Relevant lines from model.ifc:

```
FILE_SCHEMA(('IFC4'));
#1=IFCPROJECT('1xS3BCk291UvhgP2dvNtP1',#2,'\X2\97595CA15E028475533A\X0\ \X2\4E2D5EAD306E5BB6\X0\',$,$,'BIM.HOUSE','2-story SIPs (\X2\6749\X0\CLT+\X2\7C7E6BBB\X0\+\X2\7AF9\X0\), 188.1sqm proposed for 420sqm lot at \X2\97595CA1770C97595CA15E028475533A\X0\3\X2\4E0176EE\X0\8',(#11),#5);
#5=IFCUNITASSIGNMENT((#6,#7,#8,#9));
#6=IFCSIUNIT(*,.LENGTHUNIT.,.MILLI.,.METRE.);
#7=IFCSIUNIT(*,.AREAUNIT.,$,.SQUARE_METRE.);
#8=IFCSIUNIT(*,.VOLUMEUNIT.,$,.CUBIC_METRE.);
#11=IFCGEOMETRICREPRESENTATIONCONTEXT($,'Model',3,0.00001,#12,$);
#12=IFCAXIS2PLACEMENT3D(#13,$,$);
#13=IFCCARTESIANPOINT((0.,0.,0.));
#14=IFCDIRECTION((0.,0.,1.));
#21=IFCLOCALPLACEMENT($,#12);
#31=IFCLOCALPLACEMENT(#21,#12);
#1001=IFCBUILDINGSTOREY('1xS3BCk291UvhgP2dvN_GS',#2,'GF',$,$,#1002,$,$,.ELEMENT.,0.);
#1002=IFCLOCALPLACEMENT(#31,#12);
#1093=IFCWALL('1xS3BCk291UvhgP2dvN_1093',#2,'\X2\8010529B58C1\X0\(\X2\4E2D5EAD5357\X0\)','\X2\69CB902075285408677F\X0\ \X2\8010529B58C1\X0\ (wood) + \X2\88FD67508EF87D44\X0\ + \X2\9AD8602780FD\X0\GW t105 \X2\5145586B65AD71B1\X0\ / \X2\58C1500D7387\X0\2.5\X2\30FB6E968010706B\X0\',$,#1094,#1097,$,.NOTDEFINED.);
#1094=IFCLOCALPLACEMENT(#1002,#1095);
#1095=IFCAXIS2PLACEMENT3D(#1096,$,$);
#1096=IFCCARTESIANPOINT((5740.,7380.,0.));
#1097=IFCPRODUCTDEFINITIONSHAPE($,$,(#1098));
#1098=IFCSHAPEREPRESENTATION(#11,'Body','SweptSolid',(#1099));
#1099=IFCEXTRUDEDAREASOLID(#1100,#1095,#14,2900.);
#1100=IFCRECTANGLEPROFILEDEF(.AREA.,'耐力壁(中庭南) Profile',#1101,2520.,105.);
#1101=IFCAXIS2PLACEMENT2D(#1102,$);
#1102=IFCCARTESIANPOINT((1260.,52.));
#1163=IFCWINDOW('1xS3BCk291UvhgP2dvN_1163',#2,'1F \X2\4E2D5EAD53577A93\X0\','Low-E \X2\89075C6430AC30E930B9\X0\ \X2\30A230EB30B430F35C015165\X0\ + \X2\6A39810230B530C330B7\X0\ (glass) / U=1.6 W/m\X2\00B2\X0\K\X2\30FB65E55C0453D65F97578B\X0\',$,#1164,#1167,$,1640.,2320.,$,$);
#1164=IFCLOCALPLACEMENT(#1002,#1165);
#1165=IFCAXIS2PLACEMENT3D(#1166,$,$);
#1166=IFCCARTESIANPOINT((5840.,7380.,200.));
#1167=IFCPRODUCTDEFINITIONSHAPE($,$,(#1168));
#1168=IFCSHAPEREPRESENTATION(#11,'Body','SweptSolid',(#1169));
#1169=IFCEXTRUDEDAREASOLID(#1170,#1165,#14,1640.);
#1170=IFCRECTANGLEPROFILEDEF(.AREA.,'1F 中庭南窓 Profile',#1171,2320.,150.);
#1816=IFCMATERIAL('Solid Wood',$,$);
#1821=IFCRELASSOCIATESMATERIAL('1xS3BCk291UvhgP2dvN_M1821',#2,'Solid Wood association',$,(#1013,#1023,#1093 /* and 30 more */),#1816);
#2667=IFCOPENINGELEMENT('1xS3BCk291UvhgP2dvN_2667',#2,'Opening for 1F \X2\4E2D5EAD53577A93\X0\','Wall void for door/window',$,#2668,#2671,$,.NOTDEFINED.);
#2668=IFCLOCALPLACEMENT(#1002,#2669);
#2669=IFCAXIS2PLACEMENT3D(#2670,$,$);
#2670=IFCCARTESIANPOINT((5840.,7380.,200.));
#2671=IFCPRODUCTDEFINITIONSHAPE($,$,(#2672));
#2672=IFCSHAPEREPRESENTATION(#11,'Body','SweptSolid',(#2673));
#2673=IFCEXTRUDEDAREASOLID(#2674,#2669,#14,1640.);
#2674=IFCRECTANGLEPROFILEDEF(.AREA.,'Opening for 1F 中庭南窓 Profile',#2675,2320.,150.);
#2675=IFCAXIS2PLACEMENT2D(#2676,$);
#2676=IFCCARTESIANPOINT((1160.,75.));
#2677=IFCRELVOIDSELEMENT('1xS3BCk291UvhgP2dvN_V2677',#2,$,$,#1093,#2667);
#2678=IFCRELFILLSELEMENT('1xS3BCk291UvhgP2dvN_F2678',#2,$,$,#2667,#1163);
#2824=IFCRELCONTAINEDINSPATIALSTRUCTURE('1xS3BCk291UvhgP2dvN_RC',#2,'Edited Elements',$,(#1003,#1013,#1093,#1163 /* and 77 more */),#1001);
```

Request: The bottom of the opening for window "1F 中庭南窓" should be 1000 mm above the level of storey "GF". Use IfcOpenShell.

```python
import numpy as np
import ifcopenshell
import ifcopenshell.api.geometry
import ifcopenshell.geom
import ifcopenshell.util.element
import ifcopenshell.util.placement
import ifcopenshell.util.shape
import ifcopenshell.util.unit

model = ifcopenshell.open("model.ifc")
unit_scale = ifcopenshell.util.unit.calculate_unit_scale(model)

window = model.by_guid("1xS3BCk291UvhgP2dvN_1163")
opening = window.FillsVoids[0].RelatingOpeningElement
storey = ifcopenshell.util.element.get_container(window, ifc_class="IfcBuildingStorey")
level = ifcopenshell.util.placement.get_local_placement(storey.ObjectPlacement)[2, 3]

# The opening's origin need not be at the sill, so measure its lowest point.
shape = ifcopenshell.geom.create_shape(ifcopenshell.geom.settings(), opening)
bottom = ifcopenshell.util.shape.get_shape_bottom_elevation(shape, shape.geometry) / unit_scale
dz = level + 1000.0 - bottom

shift = np.array([0.0, 0.0, dz])
# The window is not placed relative to its opening, so move both.
for product in (opening, window):
    matrix = ifcopenshell.util.placement.get_local_placement(product.ObjectPlacement)
    matrix[:3, 3] += shift
    ifcopenshell.api.geometry.edit_object_placement(model, product=product, matrix=matrix, is_si=False)

print(f"moved by {dz * unit_scale:+.3f} m")

model.write("model-out.ifc")
```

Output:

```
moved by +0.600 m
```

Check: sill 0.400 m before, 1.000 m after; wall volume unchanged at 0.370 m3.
